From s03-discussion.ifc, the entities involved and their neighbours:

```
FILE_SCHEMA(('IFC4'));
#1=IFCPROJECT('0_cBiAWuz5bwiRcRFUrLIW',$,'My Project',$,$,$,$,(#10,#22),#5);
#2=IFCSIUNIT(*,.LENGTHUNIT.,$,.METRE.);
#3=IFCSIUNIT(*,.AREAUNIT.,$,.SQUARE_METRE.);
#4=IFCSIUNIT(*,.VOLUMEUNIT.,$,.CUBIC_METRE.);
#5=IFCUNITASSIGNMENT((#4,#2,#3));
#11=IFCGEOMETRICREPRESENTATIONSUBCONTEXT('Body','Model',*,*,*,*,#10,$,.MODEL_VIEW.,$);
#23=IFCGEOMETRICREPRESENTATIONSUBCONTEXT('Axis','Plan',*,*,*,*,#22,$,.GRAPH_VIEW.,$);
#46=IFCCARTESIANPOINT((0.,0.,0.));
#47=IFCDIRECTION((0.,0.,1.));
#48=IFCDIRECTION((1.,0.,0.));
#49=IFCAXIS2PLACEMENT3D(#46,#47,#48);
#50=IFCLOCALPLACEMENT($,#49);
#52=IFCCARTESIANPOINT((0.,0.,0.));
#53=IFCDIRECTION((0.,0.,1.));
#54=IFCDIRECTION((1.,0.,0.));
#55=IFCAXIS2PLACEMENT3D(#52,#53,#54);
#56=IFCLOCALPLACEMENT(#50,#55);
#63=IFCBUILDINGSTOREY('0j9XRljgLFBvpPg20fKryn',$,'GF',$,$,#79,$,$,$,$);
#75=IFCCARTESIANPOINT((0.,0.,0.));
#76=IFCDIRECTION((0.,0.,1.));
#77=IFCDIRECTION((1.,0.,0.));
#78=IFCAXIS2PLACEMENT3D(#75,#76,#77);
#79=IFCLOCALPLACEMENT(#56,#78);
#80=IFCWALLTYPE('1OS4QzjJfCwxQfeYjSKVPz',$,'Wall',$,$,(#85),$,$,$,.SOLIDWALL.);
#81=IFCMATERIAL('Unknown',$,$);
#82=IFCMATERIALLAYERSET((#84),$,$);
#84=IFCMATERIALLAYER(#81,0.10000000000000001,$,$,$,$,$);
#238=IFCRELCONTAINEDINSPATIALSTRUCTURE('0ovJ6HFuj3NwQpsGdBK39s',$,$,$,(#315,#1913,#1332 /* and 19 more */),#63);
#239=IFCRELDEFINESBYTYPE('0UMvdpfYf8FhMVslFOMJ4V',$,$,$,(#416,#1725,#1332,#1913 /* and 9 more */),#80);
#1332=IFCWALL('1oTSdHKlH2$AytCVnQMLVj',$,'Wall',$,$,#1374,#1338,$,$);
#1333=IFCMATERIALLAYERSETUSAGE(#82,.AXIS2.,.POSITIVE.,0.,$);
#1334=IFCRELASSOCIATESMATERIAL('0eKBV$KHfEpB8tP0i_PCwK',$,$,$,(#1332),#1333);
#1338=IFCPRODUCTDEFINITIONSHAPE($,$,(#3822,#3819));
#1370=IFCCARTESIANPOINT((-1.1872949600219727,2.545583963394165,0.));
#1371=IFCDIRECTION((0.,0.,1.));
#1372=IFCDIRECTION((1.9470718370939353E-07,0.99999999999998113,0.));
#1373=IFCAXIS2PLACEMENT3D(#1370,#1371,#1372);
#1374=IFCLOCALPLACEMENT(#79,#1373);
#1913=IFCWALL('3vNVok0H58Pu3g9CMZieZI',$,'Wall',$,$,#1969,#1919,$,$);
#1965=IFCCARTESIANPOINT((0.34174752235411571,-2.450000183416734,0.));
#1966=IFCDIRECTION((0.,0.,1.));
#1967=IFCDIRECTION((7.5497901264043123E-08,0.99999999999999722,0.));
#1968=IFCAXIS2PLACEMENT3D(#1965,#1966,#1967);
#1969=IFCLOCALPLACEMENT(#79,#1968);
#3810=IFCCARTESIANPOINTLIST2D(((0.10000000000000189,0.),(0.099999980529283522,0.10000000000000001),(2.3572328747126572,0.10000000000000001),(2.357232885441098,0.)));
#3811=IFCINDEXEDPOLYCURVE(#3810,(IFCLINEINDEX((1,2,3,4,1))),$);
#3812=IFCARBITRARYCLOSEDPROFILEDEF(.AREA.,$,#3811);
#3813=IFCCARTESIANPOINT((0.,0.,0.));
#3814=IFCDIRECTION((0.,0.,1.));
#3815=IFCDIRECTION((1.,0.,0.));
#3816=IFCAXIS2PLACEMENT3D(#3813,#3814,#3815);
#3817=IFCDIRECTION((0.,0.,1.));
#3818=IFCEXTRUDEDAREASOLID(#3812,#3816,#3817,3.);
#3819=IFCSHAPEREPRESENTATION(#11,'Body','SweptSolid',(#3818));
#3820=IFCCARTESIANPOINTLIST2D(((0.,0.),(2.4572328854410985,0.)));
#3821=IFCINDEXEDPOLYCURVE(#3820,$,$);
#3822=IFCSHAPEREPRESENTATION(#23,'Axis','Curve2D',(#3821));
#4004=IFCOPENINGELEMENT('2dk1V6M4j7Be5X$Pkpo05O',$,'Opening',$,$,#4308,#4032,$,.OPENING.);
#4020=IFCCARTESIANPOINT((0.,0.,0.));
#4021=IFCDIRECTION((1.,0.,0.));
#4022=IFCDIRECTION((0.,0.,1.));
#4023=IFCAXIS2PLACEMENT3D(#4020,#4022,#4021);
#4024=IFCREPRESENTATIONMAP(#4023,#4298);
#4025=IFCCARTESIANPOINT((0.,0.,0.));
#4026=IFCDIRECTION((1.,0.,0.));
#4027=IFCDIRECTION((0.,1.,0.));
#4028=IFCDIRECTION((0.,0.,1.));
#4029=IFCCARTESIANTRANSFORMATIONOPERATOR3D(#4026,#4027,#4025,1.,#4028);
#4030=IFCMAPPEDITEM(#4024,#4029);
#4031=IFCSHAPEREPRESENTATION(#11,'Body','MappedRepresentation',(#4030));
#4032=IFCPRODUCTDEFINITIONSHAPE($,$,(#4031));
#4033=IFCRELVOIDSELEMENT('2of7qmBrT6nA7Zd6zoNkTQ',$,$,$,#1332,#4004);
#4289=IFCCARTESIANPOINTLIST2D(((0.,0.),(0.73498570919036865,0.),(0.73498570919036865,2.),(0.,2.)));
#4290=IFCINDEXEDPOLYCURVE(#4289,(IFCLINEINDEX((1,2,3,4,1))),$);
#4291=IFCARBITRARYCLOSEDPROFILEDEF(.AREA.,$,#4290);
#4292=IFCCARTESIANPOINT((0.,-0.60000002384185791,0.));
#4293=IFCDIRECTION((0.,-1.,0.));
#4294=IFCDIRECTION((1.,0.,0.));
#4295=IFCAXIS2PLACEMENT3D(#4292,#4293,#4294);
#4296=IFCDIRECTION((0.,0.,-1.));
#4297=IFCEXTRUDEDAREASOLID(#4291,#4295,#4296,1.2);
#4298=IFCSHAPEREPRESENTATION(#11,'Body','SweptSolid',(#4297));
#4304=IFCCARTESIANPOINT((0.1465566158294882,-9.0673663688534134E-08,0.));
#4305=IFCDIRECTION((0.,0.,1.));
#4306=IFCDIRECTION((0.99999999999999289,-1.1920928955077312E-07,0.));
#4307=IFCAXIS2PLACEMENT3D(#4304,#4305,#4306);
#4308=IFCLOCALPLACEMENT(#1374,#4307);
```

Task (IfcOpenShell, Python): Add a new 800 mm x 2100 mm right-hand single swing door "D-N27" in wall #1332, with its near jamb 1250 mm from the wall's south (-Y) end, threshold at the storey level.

```python
import numpy as np
import ifcopenshell
import ifcopenshell.api.feature
import ifcopenshell.api.geometry
import ifcopenshell.api.root
import ifcopenshell.api.spatial
import ifcopenshell.geom
import ifcopenshell.util.element
import ifcopenshell.util.placement
import ifcopenshell.util.representation
import ifcopenshell.util.shape
import ifcopenshell.util.unit

model = ifcopenshell.open("s03-discussion.ifc")
unit_scale = ifcopenshell.util.unit.calculate_unit_scale(model)
settings = ifcopenshell.geom.settings()


def volume(element):
    """Net volume in cubic metres, openings subtracted."""
    shape = ifcopenshell.geom.create_shape(settings, element)
    return ifcopenshell.util.shape.get_volume(shape.geometry)


wall = model.by_guid("1oTSdHKlH2$AytCVnQMLVj")
storey = ifcopenshell.util.element.get_container(wall, ifc_class="IfcBuildingStorey")
context = ifcopenshell.util.representation.get_context(model, "Model", "Body", "MODEL_VIEW")
before = volume(wall)

width, height, from_end, sill = 0.8, 2.1, 1.25, 0.0  # metres

# The wall runs along its own X axis, and the end named is its -X end.
wall_shape = ifcopenshell.geom.create_shape(settings, wall)
x, y, z = ifcopenshell.util.shape.get_vertices(wall_shape.geometry).T
start = x.min() + from_end
face, thickness = float(y.min()), float(y.max() - y.min())
wall_matrix = ifcopenshell.util.placement.get_local_placement(wall.ObjectPlacement)
level = ifcopenshell.util.placement.get_local_placement(storey.ObjectPlacement)[2, 3]


def in_wall(x, y):
    """Placement at x, y metres in the wall's axes, at sill height."""
    matrix = wall_matrix.copy()
    matrix[:, 3] = wall_matrix @ np.array([x / unit_scale, y / unit_scale, 0.0, 1.0])
    matrix[2, 3] = level + sill / unit_scale
    return matrix


# Opening: a box that overshoots both wall faces by 50 mm.
opening = ifcopenshell.api.root.create_entity(model, ifc_class="IfcOpeningElement", predefined_type="OPENING")
box = ifcopenshell.api.geometry.add_wall_representation(
    model, context=context, length=width, height=height, thickness=thickness + 0.1
)
ifcopenshell.api.geometry.assign_representation(model, product=opening, representation=box)
ifcopenshell.api.geometry.edit_object_placement(model, product=opening, matrix=in_wall(start, face - 0.05), is_si=False)
ifcopenshell.api.feature.add_feature(model, feature=opening, element=wall)

door = ifcopenshell.api.root.create_entity(model, ifc_class="IfcDoor", name="D-N27", predefined_type="DOOR")
door.OverallWidth, door.OverallHeight = width / unit_scale, height / unit_scale
door.OperationType = "SINGLE_SWING_RIGHT"
body = ifcopenshell.api.geometry.add_door_representation(
    model,
    context=context,
    overall_width=door.OverallWidth,
    overall_height=door.OverallHeight,
    operation_type="SINGLE_SWING_RIGHT",
    lining_properties={"LiningDepth": thickness / unit_scale, "ThresholdDepth": thickness / unit_scale},
)
ifcopenshell.api.geometry.assign_representation(model, product=door, representation=body)
ifcopenshell.api.spatial.assign_container(model, products=[door], relating_structure=storey)
ifcopenshell.api.feature.add_filling(model, opening=opening, element=door)

# The lining spans the wall, so the door starts at the wall face.
ifcopenshell.api.geometry.edit_object_placement(model, product=door, matrix=in_wall(start, face), is_si=False)

after = volume(wall)

print(f"wall volume {before:.3f} -> {after:.3f} m3")

model.write("s03-discussion_edited.ifc")
```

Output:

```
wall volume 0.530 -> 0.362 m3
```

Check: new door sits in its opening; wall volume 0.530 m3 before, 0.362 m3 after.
